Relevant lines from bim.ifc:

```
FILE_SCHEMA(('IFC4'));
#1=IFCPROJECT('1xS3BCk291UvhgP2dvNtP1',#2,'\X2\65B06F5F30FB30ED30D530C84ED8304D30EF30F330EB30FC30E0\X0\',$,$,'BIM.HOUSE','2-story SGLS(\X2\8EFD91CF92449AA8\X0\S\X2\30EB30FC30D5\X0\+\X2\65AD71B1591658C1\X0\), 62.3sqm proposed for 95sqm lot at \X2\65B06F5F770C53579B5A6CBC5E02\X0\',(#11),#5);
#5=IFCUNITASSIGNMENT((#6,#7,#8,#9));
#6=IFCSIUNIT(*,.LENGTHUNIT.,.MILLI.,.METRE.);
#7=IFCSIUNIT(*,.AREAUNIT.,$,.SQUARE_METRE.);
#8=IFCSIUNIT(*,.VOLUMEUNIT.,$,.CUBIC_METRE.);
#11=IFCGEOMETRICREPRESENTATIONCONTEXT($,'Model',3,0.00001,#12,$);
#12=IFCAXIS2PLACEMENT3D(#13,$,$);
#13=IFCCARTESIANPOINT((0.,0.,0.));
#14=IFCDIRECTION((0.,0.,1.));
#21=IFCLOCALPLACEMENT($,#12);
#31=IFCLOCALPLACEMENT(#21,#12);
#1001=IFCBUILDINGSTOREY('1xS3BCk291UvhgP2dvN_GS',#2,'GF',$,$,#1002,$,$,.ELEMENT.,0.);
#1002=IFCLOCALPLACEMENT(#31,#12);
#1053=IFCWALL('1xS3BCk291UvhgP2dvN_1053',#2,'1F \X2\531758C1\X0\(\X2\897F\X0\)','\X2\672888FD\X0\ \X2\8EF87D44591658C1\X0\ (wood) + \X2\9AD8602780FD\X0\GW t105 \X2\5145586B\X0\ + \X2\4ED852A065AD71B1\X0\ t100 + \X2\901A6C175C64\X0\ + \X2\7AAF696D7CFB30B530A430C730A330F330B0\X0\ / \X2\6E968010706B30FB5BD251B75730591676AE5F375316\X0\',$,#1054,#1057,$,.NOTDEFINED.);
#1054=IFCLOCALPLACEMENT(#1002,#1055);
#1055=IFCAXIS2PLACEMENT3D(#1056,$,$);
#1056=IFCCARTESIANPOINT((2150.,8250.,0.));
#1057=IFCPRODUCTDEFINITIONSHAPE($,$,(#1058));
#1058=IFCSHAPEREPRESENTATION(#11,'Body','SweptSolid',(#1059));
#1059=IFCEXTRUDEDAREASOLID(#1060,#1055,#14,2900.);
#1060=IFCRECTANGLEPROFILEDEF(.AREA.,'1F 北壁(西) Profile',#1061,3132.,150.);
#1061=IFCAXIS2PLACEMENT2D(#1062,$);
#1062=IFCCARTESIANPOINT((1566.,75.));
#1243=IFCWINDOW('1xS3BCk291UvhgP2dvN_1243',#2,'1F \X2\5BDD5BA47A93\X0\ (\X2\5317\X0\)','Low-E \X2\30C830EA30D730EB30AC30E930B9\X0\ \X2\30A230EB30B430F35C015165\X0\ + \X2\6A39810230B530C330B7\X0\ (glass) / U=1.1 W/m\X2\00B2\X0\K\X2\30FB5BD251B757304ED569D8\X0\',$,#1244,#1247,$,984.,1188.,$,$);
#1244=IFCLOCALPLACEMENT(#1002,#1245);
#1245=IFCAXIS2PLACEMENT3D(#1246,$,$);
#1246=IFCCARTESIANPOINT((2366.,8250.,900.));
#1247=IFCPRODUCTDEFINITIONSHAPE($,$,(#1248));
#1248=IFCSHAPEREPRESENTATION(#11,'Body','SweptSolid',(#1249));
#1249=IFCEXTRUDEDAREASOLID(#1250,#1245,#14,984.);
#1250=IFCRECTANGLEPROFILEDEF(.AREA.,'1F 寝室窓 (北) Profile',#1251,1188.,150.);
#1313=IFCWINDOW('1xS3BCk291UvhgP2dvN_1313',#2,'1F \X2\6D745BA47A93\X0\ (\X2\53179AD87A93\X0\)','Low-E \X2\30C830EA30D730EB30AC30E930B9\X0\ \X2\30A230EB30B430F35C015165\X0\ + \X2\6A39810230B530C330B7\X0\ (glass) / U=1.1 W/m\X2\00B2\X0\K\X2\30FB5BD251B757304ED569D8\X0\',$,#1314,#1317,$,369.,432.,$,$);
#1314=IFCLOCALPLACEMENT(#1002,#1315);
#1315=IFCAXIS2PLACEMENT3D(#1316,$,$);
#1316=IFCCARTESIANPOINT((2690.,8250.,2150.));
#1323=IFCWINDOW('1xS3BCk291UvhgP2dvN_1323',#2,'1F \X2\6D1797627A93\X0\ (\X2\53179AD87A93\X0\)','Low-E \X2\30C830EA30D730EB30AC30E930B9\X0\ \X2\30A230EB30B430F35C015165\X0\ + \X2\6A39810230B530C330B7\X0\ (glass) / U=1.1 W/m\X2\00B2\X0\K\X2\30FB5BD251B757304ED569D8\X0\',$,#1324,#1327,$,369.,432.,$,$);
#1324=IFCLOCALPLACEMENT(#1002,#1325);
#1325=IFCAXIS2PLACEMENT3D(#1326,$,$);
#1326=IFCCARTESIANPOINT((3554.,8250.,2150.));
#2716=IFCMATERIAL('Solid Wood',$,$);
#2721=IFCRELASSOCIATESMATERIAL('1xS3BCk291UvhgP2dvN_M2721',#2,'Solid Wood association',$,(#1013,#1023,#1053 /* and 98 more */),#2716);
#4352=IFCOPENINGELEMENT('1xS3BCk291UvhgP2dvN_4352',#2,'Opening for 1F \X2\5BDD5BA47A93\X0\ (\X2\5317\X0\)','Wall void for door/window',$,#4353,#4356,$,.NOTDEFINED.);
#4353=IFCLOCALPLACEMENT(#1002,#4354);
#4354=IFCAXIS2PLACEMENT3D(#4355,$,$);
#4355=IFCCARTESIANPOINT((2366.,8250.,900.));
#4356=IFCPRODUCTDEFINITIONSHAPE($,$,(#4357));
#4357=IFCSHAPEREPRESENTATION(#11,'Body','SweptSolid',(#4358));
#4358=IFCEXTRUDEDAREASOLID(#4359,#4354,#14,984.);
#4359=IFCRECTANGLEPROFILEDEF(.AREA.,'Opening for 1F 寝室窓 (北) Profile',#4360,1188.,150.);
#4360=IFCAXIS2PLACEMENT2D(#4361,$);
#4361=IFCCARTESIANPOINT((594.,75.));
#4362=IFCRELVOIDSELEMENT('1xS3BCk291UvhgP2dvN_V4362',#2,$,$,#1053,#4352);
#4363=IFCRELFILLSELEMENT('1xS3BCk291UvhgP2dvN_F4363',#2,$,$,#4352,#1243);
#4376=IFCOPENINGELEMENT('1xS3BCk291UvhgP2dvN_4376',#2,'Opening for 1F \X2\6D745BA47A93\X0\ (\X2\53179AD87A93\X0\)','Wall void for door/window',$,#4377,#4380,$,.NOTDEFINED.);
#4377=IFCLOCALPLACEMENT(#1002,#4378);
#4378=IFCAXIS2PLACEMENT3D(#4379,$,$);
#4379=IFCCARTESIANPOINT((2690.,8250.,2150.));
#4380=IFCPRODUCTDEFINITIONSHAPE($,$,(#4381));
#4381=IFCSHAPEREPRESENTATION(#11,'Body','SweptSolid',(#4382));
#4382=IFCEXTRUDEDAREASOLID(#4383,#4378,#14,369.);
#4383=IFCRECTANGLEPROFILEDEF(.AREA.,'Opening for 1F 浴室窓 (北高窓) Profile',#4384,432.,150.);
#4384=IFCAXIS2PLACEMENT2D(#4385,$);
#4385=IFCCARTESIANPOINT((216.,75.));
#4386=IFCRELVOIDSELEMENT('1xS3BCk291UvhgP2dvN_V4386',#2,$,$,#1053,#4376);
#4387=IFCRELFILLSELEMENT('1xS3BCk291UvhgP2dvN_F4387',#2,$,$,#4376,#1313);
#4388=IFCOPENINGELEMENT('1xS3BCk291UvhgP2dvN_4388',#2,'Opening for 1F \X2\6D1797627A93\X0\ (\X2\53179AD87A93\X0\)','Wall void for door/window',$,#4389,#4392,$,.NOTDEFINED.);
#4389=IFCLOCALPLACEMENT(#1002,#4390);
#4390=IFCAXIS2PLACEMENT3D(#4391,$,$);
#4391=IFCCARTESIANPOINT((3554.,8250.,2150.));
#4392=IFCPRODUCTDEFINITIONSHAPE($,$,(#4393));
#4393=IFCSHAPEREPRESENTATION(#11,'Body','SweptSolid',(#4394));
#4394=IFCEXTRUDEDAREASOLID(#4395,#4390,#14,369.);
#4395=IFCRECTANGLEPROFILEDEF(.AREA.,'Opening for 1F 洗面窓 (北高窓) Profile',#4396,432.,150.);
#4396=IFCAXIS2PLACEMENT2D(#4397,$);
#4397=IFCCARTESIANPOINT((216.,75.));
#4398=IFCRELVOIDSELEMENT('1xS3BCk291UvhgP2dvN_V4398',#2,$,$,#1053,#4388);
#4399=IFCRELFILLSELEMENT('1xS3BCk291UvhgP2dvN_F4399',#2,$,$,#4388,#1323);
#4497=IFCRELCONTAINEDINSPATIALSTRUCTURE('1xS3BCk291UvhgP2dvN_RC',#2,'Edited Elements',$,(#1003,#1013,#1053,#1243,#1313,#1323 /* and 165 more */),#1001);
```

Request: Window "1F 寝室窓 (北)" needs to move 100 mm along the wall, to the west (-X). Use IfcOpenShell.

```python
import ifcopenshell
import ifcopenshell.api.geometry
import ifcopenshell.util.placement
import ifcopenshell.util.unit

model = ifcopenshell.open("bim.ifc")
unit_scale = ifcopenshell.util.unit.calculate_unit_scale(model)

window = model.by_id(1243)
opening = window.FillsVoids[0].RelatingOpeningElement
wall = opening.VoidsElements[0].RelatingBuildingElement

wall_matrix = ifcopenshell.util.placement.get_local_placement(wall.ObjectPlacement)
shift = wall_matrix[:3, 0] * -0.1 / unit_scale
before = ifcopenshell.util.placement.get_local_placement(window.ObjectPlacement)[:3, 3].copy()

# The window is not placed relative to its opening, so move both.
for product in (opening, window):
    matrix = ifcopenshell.util.placement.get_local_placement(product.ObjectPlacement)
    matrix[:3, 3] += shift
    ifcopenshell.api.geometry.edit_object_placement(model, product=product, matrix=matrix, is_si=False)

after = ifcopenshell.util.placement.get_local_placement(window.ObjectPlacement)[:3, 3]
print("window moved by", (after - before).round(3) + 0.0)

model.write("bim-out.ifc")
```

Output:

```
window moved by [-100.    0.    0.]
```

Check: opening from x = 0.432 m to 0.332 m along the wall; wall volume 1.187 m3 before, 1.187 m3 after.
